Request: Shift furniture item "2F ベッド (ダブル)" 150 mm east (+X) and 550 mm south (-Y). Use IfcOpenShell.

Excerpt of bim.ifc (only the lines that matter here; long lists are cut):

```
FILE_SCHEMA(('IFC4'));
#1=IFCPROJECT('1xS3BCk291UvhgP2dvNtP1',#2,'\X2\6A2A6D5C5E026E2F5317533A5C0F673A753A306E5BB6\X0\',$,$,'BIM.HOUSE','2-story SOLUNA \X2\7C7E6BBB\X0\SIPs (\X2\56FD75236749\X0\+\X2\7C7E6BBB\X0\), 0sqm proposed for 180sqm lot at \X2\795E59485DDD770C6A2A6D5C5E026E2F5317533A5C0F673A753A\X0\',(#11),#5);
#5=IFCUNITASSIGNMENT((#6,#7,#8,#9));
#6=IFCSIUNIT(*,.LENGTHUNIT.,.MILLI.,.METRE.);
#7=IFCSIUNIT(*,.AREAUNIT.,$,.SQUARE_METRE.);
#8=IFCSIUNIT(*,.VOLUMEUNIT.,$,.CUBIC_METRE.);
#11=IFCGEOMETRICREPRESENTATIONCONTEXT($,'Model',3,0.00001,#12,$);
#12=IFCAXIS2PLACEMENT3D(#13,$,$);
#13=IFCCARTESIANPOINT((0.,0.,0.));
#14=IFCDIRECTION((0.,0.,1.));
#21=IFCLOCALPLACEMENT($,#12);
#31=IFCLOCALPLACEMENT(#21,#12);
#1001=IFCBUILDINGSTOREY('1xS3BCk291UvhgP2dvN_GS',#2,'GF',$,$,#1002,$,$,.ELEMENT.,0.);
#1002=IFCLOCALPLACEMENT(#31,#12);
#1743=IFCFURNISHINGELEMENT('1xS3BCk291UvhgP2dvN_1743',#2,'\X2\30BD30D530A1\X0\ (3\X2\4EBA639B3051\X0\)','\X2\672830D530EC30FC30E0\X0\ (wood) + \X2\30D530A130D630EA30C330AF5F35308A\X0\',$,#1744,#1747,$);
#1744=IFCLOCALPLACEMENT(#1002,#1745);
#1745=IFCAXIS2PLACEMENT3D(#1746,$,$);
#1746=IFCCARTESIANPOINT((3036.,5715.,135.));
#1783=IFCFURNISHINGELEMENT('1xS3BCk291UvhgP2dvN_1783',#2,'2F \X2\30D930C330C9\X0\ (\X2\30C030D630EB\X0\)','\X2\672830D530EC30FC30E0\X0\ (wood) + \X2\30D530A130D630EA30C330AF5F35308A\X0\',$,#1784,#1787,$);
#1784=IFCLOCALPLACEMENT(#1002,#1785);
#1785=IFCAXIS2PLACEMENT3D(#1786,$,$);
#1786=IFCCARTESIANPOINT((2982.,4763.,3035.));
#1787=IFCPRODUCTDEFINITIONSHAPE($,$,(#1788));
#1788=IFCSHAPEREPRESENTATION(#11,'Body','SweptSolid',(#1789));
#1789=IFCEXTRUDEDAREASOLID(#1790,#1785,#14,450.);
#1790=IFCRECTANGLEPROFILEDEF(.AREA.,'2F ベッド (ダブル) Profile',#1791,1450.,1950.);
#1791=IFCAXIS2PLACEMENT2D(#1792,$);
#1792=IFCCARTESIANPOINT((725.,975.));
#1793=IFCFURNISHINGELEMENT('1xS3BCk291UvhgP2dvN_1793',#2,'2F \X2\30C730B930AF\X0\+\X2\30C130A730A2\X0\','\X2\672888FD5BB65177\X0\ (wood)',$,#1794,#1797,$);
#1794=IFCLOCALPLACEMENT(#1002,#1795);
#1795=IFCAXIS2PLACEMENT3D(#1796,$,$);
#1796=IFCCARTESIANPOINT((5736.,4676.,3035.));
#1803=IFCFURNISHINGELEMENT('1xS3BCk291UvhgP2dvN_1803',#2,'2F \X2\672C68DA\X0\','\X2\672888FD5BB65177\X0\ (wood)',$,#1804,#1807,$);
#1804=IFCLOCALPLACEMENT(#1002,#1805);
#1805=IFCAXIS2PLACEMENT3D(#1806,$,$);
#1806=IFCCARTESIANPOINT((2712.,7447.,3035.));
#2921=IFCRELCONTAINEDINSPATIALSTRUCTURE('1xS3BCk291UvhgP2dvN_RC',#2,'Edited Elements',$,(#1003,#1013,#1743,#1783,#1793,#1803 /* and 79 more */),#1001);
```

```python
import ifcopenshell
import ifcopenshell.api.geometry
import ifcopenshell.util.placement
import ifcopenshell.util.unit

model = ifcopenshell.open("bim.ifc")
unit_scale = ifcopenshell.util.unit.calculate_unit_scale(model)

item = model.by_guid("1xS3BCk291UvhgP2dvN_1783")
matrix = ifcopenshell.util.placement.get_local_placement(item.ObjectPlacement)
matrix[0, 3] += 0.15 / unit_scale
matrix[1, 3] -= 0.55 / unit_scale
ifcopenshell.api.geometry.edit_object_placement(model, product=item, matrix=matrix, is_si=False)

print(ifcopenshell.util.placement.get_local_placement(item.ObjectPlacement).round(3) + 0.0)

model.write("bim-out.ifc")
```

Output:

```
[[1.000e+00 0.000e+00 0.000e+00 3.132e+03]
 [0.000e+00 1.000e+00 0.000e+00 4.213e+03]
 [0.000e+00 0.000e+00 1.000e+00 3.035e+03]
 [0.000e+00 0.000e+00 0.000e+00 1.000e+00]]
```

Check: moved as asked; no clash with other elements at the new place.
